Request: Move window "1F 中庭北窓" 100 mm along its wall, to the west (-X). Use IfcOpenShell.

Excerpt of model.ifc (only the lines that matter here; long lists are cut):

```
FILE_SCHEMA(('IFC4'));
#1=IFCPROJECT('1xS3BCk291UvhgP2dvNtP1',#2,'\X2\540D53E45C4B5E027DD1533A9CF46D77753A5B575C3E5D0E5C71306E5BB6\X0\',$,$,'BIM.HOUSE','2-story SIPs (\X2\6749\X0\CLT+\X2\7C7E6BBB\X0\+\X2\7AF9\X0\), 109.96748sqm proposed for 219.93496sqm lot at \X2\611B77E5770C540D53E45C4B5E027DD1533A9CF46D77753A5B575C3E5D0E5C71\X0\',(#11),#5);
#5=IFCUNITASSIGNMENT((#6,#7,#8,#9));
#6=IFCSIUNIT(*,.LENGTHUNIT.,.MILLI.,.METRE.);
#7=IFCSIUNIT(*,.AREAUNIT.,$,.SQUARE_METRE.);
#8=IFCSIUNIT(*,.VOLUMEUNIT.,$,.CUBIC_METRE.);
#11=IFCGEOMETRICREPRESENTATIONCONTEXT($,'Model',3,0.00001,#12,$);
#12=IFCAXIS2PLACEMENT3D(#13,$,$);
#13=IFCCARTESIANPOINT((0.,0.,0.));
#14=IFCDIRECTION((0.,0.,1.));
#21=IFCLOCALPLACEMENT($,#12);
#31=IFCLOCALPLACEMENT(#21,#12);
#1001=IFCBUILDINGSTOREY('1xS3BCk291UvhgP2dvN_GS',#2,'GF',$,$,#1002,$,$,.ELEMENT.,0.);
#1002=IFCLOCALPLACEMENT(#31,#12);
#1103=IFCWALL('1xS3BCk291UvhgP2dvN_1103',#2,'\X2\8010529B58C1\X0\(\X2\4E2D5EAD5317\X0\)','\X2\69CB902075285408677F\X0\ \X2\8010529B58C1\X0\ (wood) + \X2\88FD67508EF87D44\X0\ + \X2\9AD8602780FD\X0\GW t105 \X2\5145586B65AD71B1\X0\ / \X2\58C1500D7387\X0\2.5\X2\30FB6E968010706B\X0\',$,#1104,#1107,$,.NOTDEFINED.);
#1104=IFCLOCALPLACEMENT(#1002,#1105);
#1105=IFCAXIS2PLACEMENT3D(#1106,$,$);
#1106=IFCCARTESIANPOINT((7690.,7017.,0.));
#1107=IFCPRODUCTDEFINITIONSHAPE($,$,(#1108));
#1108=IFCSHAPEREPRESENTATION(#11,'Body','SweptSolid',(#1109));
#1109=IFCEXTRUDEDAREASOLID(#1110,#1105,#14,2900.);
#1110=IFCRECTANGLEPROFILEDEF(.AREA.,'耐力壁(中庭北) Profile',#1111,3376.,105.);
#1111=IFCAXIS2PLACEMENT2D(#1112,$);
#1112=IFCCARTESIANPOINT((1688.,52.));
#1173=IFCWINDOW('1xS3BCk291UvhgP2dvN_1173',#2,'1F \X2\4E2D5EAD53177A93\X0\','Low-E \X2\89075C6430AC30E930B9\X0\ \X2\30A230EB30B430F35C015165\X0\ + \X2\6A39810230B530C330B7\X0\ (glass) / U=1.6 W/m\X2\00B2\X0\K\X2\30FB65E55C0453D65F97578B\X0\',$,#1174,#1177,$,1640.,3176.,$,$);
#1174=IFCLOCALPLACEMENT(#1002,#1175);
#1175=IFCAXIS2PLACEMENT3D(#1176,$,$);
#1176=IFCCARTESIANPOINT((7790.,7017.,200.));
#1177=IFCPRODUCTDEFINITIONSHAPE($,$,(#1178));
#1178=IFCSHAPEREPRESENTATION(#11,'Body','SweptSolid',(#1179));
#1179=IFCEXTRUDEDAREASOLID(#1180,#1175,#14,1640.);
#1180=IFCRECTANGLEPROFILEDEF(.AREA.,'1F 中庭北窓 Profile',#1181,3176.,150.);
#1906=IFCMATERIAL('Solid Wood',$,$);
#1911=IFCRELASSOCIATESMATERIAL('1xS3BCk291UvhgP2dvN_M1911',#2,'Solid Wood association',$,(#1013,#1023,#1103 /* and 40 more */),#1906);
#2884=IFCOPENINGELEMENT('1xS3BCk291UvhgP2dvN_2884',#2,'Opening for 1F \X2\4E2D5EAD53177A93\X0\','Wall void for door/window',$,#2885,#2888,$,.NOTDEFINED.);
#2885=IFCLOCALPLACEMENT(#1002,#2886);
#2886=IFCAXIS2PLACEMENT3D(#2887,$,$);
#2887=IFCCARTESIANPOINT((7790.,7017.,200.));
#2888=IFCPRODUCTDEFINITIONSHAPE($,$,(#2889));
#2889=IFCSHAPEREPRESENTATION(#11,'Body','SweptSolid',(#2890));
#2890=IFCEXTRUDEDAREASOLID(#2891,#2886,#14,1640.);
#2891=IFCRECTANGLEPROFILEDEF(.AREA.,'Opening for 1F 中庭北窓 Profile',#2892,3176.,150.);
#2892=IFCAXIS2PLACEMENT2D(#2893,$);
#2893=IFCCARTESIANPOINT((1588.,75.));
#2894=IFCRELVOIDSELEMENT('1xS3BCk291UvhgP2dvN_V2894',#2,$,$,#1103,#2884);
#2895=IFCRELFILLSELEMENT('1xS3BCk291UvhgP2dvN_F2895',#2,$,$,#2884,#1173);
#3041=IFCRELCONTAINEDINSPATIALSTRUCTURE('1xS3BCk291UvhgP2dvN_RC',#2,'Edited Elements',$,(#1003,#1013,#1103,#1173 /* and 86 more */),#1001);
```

```python
import ifcopenshell
import ifcopenshell.api.geometry
import ifcopenshell.util.placement
import ifcopenshell.util.unit

model = ifcopenshell.open("model.ifc")
unit_scale = ifcopenshell.util.unit.calculate_unit_scale(model)

window = model.by_id(1173)
opening = window.FillsVoids[0].RelatingOpeningElement
wall = opening.VoidsElements[0].RelatingBuildingElement

wall_matrix = ifcopenshell.util.placement.get_local_placement(wall.ObjectPlacement)
shift = wall_matrix[:3, 0] * -0.1 / unit_scale
before = ifcopenshell.util.placement.get_local_placement(window.ObjectPlacement)[:3, 3].copy()

# The window is not placed relative to its opening, so move both.
for product in (opening, window):
    matrix = ifcopenshell.util.placement.get_local_placement(product.ObjectPlacement)
    matrix[:3, 3] += shift
    ifcopenshell.api.geometry.edit_object_placement(model, product=product, matrix=matrix, is_si=False)

after = ifcopenshell.util.placement.get_local_placement(window.ObjectPlacement)[:3, 3]
print("window moved by", (after - before).round(3) + 0.0)

model.write("model-out.ifc")
```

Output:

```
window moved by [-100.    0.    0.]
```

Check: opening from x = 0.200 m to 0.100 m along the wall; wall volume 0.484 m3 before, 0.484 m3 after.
